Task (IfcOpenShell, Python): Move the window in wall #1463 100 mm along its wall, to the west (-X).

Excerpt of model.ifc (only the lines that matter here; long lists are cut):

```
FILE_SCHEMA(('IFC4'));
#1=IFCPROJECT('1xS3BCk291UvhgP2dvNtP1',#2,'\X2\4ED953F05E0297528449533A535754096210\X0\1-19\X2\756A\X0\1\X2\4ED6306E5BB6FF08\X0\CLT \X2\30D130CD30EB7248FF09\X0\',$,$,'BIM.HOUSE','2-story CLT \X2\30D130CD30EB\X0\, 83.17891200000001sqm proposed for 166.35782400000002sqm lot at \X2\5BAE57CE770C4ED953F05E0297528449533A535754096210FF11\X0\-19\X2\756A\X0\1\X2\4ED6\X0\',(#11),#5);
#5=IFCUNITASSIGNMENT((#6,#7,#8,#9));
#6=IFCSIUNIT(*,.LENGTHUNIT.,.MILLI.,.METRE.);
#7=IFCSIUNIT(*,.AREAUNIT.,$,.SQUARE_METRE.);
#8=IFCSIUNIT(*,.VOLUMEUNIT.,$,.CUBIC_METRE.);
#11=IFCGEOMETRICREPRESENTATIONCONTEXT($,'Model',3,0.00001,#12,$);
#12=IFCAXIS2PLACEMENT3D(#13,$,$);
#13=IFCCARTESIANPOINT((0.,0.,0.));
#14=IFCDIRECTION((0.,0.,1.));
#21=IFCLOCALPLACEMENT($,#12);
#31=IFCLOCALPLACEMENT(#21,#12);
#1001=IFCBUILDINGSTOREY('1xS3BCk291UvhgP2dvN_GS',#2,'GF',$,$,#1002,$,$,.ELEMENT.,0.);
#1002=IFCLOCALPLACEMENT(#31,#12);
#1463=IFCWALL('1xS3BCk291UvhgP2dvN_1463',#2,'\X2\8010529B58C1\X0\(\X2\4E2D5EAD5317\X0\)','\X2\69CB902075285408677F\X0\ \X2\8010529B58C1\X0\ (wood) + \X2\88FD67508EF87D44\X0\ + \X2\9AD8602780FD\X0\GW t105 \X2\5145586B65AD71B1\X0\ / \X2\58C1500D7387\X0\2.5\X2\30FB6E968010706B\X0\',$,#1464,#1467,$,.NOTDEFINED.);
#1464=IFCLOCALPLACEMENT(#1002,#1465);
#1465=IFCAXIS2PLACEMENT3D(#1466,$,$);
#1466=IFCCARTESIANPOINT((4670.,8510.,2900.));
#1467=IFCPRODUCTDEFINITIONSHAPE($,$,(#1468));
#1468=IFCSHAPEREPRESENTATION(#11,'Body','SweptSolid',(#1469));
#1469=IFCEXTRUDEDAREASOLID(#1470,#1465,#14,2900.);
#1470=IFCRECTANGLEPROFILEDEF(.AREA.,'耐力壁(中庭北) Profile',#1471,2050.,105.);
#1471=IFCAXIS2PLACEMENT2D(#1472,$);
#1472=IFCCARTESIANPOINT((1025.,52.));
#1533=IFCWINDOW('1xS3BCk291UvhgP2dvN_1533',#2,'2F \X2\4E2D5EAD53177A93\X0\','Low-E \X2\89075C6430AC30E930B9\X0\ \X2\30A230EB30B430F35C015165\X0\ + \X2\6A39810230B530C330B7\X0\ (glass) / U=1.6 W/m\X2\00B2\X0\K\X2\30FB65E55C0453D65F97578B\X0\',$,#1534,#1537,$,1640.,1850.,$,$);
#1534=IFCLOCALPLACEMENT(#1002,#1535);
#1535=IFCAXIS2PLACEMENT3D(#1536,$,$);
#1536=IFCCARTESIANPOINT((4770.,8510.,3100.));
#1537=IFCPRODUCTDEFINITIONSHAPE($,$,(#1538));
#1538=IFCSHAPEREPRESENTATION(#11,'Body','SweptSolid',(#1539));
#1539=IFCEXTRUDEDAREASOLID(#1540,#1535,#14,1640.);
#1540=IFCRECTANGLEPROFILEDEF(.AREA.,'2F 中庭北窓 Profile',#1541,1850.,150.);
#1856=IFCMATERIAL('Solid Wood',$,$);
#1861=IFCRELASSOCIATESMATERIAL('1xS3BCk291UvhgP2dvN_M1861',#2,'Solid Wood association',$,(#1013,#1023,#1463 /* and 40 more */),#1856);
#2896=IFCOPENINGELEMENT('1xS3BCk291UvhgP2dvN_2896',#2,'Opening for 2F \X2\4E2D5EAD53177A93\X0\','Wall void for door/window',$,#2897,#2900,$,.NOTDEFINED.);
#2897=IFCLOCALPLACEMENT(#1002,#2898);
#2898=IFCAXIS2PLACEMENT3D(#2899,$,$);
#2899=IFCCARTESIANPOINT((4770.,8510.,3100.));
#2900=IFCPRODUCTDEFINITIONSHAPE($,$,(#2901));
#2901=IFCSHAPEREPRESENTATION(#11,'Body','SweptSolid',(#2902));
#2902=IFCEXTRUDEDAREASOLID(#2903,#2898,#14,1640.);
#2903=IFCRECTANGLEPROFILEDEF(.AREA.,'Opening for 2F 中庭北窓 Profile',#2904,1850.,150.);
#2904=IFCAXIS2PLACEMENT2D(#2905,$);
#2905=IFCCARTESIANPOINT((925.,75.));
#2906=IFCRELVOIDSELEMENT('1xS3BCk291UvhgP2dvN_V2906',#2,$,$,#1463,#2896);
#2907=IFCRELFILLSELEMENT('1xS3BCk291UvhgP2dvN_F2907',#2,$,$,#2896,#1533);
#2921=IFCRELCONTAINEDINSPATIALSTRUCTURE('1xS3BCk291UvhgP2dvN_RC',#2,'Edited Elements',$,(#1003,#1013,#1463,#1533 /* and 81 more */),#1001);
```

```python
import ifcopenshell
import ifcopenshell.api.geometry
import ifcopenshell.util.placement
import ifcopenshell.util.unit

model = ifcopenshell.open("model.ifc")
unit_scale = ifcopenshell.util.unit.calculate_unit_scale(model)

window = model.by_id(1533)
opening = window.FillsVoids[0].RelatingOpeningElement
wall = opening.VoidsElements[0].RelatingBuildingElement

wall_matrix = ifcopenshell.util.placement.get_local_placement(wall.ObjectPlacement)
shift = wall_matrix[:3, 0] * -0.1 / unit_scale
before = ifcopenshell.util.placement.get_local_placement(window.ObjectPlacement)[:3, 3].copy()

# The window is not placed relative to its opening, so move both.
for product in (opening, window):
    matrix = ifcopenshell.util.placement.get_local_placement(product.ObjectPlacement)
    matrix[:3, 3] += shift
    ifcopenshell.api.geometry.edit_object_placement(model, product=product, matrix=matrix, is_si=False)

after = ifcopenshell.util.placement.get_local_placement(window.ObjectPlacement)[:3, 3]
print("window moved by", (after - before).round(3) + 0.0)

model.write("model_v2.ifc")
```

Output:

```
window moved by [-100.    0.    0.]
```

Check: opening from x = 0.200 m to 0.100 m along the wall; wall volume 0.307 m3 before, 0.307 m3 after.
